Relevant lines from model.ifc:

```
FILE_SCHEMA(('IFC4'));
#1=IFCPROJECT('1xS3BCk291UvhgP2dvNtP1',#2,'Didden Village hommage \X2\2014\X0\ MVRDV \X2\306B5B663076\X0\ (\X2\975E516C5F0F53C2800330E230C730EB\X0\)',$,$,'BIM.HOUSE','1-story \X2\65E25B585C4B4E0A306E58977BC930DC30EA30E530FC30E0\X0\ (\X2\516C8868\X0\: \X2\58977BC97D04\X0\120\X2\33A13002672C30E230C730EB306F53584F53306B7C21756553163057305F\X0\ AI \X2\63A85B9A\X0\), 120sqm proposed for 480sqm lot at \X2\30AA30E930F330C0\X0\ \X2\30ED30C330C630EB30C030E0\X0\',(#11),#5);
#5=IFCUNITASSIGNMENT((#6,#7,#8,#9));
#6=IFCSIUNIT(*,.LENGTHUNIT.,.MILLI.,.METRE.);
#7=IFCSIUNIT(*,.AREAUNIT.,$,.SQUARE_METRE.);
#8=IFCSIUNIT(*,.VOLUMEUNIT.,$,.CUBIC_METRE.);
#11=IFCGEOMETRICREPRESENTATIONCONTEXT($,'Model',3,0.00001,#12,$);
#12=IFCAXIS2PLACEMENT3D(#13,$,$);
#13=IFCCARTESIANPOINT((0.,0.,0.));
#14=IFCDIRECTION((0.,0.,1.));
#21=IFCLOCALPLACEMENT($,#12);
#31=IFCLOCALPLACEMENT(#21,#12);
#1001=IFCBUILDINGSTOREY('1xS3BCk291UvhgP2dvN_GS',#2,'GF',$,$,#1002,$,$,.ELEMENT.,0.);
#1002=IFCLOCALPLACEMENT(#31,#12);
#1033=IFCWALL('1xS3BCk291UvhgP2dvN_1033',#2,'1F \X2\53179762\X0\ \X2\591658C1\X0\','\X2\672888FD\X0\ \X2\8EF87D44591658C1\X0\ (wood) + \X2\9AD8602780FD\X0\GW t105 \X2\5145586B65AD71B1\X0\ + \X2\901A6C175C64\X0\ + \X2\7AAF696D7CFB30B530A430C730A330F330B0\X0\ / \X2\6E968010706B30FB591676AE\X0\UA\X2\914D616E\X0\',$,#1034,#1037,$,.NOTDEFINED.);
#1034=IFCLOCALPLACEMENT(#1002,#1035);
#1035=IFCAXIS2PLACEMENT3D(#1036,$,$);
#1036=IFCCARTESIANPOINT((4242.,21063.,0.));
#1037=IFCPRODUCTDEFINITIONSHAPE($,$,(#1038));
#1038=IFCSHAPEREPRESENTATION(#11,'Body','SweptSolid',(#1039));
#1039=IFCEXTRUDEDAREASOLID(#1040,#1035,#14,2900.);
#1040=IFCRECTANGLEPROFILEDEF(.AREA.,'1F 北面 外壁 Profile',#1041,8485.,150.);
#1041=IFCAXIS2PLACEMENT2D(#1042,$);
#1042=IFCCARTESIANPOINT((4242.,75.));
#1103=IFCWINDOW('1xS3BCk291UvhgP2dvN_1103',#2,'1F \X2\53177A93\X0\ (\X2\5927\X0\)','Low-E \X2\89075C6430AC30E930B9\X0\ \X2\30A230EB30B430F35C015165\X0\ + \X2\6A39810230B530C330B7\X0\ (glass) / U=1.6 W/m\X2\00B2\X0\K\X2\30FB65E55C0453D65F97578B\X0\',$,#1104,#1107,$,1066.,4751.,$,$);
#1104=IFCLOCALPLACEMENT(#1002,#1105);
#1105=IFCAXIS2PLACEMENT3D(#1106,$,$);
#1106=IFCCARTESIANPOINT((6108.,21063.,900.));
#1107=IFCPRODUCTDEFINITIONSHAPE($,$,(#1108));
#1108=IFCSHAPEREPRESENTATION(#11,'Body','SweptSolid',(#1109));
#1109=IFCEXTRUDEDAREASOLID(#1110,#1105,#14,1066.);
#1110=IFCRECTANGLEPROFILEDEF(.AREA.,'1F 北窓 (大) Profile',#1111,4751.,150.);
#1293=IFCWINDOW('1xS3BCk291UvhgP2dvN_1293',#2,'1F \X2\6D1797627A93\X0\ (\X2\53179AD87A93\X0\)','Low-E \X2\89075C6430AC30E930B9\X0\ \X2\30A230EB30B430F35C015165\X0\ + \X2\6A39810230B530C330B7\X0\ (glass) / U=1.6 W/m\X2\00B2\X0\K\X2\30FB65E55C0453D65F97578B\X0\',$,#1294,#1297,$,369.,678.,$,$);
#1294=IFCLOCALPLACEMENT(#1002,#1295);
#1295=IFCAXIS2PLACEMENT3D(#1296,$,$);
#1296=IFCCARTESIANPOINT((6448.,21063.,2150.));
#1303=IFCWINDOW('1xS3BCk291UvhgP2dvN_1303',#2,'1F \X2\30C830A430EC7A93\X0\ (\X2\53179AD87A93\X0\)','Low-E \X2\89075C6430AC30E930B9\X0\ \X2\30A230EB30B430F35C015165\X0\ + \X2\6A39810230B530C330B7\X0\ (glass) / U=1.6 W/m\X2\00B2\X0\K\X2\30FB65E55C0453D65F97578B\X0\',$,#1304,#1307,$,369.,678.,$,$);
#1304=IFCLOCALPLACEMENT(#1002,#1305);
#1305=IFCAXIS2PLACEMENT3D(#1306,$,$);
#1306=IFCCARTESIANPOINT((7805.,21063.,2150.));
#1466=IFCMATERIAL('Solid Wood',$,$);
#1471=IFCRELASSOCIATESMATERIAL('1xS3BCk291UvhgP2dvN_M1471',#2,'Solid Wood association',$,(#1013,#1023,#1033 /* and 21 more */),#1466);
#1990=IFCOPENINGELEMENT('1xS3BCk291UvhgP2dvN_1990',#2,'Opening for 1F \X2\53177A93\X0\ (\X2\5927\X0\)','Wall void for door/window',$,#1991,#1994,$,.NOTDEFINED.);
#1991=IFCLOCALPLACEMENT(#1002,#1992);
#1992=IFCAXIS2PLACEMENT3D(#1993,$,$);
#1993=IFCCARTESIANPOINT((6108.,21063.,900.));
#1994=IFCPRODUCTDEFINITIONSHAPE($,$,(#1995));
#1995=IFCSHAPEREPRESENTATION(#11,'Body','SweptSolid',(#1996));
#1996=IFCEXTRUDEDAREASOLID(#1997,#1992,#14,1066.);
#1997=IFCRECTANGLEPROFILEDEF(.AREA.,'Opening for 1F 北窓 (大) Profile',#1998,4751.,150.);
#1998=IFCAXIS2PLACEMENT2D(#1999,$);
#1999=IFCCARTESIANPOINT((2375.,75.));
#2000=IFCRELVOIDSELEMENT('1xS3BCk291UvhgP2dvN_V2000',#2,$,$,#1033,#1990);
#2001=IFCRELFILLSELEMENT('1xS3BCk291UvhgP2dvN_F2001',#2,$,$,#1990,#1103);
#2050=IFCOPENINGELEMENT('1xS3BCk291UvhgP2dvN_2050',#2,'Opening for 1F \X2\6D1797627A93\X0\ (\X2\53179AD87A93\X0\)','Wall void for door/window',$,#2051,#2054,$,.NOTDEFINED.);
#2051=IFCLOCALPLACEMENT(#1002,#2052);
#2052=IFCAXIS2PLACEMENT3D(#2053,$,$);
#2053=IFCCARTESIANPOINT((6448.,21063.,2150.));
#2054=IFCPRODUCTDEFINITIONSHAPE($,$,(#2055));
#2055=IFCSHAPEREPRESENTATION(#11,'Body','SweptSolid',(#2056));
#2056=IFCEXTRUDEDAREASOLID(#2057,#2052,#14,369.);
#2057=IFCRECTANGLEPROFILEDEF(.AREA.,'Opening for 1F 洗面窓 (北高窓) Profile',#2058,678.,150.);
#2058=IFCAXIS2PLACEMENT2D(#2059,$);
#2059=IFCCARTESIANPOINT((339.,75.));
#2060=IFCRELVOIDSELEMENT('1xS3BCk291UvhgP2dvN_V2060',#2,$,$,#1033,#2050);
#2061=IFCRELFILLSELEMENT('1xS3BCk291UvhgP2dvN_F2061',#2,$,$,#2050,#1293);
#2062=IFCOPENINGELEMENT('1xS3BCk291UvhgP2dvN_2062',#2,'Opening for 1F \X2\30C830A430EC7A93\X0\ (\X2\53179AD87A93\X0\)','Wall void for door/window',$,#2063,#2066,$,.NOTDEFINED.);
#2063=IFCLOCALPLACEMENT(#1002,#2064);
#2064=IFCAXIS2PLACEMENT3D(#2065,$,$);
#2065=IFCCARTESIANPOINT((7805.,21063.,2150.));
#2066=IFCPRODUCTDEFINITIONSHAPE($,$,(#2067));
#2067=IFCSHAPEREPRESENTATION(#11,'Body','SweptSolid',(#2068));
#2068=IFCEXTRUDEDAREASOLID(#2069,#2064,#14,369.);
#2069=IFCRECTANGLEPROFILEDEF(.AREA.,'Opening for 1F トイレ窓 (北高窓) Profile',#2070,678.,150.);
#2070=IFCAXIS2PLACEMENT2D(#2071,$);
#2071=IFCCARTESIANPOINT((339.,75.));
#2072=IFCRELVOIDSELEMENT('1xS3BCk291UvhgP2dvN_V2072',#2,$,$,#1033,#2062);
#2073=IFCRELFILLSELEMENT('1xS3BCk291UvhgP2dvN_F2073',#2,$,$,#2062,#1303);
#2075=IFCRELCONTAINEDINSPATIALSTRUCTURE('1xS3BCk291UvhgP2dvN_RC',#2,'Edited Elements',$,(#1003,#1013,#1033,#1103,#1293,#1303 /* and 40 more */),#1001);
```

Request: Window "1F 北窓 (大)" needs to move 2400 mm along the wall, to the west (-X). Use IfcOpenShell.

```python
import ifcopenshell
import ifcopenshell.api.geometry
import ifcopenshell.util.placement
import ifcopenshell.util.unit

model = ifcopenshell.open("model.ifc")
unit_scale = ifcopenshell.util.unit.calculate_unit_scale(model)

window = model.by_guid("1xS3BCk291UvhgP2dvN_1103")
opening = window.FillsVoids[0].RelatingOpeningElement
wall = opening.VoidsElements[0].RelatingBuildingElement

wall_matrix = ifcopenshell.util.placement.get_local_placement(wall.ObjectPlacement)
shift = wall_matrix[:3, 0] * -2.4 / unit_scale
before = ifcopenshell.util.placement.get_local_placement(window.ObjectPlacement)[:3, 3].copy()

# The window is not placed relative to its opening, so move both.
for product in (opening, window):
    matrix = ifcopenshell.util.placement.get_local_placement(product.ObjectPlacement)
    matrix[:3, 3] += shift
    ifcopenshell.api.geometry.edit_object_placement(model, product=product, matrix=matrix, is_si=False)

after = ifcopenshell.util.placement.get_local_placement(window.ObjectPlacement)[:3, 3]
print("window moved by", (after - before).round(3) + 0.0)

model.write("model_v2.ifc")
```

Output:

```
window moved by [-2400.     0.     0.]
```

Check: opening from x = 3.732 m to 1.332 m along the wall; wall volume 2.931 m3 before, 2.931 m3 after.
